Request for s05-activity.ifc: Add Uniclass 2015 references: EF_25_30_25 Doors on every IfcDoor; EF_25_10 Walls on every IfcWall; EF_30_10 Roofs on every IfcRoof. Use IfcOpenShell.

First a look at what the model holds.

```python
import ifcopenshell

model = ifcopenshell.open("s05-activity.ifc")
print(model.schema)
print("classifications:", [c.Name for c in model.by_type("IfcClassification")])
for ifc_class in ("IfcDoor", "IfcRoof", "IfcStair", "IfcWall", "IfcWindow"):
    print(ifc_class, len(model.by_type(ifc_class)))
```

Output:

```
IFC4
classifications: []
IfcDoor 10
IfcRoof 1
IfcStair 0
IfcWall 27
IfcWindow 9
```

```python
import ifcopenshell
import ifcopenshell.api.classification

model = ifcopenshell.open("s05-activity.ifc")

system = ifcopenshell.api.classification.add_classification(model, classification="Uniclass 2015")

codes = {
    "IfcDoor": ("EF_25_30_25", "Doors"),
    "IfcWall": ("EF_25_10", "Walls"),
    "IfcRoof": ("EF_30_10", "Roofs"),
}
for ifc_class, (code, name) in codes.items():
    products = model.by_type(ifc_class)
    ifcopenshell.api.classification.add_reference(
        model, products=products, classification=system, identification=code, name=name
    )
    print(code, len(products))

model.write("s05-activity-out.ifc")
```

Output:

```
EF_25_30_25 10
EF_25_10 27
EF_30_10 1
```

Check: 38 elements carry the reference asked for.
